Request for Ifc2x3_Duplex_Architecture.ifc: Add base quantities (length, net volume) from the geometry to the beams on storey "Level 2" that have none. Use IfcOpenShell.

First a look at what the model holds.

```python
import ifcopenshell
import ifcopenshell.util.element
import ifcopenshell.util.unit

model = ifcopenshell.open("Ifc2x3_Duplex_Architecture.ifc")
print(model.schema)
for unit_type in ("LENGTHUNIT", "AREAUNIT", "VOLUMEUNIT"):
    print(unit_type, ifcopenshell.util.unit.calculate_unit_scale(model, unit_type))
storey = next(s for s in model.by_type("IfcBuildingStorey") if s.Name == "Level 2")
beams = [e for e in ifcopenshell.util.element.get_decomposition(storey) if e.is_a("IfcBeam")]
for e in sorted(beams, key=lambda e: e.id()):
    print(e.id(), e.is_a(), e.Name, list(ifcopenshell.util.element.get_psets(e, qtos_only=True)), sep=" | ")
```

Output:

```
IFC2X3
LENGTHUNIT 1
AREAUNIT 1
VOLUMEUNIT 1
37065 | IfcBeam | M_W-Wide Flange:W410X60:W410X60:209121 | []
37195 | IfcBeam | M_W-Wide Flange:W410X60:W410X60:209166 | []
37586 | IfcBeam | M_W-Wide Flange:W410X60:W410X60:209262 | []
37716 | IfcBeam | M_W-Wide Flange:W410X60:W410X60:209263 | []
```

```python
import ifcopenshell
import ifcopenshell.api.pset
import ifcopenshell.geom
import ifcopenshell.util.element
import ifcopenshell.util.shape
import ifcopenshell.util.unit

model = ifcopenshell.open("Ifc2x3_Duplex_Architecture.ifc")
unit_scale = ifcopenshell.util.unit.calculate_unit_scale(model)
volume_scale = ifcopenshell.util.unit.calculate_unit_scale(model, "VOLUMEUNIT")
settings = ifcopenshell.geom.settings()

storey = next(s for s in model.by_type("IfcBuildingStorey") if s.Name == "Level 2")
beams = [e for e in ifcopenshell.util.element.get_decomposition(storey) if e.is_a("IfcBeam")]

for e in sorted(beams, key=lambda e: e.id()):
    if ifcopenshell.util.element.get_psets(e, qtos_only=True, should_inherit=False):
        continue
    # Geometry comes back in metres, in the element's own axes.
    shape = ifcopenshell.geom.create_shape(settings, e)
    values = {
        "Length": ifcopenshell.util.shape.get_max_xyz(shape.geometry) / unit_scale,
        "NetVolume": ifcopenshell.util.shape.get_volume(shape.geometry) / volume_scale,
    }
    qto = ifcopenshell.api.pset.add_qto(model, product=e, name="BaseQuantities")
    ifcopenshell.api.pset.edit_qto(model, qto=qto, properties=values)
    print(e.id(), {k: round(v, 3) for k, v in values.items()})

model.write("Ifc2x3_Duplex_Architecture_updated.ifc")
```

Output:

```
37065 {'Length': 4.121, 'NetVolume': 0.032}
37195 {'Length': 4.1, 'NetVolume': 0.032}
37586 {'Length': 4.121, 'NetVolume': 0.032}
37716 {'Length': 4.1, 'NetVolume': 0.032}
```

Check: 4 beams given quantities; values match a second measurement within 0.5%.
